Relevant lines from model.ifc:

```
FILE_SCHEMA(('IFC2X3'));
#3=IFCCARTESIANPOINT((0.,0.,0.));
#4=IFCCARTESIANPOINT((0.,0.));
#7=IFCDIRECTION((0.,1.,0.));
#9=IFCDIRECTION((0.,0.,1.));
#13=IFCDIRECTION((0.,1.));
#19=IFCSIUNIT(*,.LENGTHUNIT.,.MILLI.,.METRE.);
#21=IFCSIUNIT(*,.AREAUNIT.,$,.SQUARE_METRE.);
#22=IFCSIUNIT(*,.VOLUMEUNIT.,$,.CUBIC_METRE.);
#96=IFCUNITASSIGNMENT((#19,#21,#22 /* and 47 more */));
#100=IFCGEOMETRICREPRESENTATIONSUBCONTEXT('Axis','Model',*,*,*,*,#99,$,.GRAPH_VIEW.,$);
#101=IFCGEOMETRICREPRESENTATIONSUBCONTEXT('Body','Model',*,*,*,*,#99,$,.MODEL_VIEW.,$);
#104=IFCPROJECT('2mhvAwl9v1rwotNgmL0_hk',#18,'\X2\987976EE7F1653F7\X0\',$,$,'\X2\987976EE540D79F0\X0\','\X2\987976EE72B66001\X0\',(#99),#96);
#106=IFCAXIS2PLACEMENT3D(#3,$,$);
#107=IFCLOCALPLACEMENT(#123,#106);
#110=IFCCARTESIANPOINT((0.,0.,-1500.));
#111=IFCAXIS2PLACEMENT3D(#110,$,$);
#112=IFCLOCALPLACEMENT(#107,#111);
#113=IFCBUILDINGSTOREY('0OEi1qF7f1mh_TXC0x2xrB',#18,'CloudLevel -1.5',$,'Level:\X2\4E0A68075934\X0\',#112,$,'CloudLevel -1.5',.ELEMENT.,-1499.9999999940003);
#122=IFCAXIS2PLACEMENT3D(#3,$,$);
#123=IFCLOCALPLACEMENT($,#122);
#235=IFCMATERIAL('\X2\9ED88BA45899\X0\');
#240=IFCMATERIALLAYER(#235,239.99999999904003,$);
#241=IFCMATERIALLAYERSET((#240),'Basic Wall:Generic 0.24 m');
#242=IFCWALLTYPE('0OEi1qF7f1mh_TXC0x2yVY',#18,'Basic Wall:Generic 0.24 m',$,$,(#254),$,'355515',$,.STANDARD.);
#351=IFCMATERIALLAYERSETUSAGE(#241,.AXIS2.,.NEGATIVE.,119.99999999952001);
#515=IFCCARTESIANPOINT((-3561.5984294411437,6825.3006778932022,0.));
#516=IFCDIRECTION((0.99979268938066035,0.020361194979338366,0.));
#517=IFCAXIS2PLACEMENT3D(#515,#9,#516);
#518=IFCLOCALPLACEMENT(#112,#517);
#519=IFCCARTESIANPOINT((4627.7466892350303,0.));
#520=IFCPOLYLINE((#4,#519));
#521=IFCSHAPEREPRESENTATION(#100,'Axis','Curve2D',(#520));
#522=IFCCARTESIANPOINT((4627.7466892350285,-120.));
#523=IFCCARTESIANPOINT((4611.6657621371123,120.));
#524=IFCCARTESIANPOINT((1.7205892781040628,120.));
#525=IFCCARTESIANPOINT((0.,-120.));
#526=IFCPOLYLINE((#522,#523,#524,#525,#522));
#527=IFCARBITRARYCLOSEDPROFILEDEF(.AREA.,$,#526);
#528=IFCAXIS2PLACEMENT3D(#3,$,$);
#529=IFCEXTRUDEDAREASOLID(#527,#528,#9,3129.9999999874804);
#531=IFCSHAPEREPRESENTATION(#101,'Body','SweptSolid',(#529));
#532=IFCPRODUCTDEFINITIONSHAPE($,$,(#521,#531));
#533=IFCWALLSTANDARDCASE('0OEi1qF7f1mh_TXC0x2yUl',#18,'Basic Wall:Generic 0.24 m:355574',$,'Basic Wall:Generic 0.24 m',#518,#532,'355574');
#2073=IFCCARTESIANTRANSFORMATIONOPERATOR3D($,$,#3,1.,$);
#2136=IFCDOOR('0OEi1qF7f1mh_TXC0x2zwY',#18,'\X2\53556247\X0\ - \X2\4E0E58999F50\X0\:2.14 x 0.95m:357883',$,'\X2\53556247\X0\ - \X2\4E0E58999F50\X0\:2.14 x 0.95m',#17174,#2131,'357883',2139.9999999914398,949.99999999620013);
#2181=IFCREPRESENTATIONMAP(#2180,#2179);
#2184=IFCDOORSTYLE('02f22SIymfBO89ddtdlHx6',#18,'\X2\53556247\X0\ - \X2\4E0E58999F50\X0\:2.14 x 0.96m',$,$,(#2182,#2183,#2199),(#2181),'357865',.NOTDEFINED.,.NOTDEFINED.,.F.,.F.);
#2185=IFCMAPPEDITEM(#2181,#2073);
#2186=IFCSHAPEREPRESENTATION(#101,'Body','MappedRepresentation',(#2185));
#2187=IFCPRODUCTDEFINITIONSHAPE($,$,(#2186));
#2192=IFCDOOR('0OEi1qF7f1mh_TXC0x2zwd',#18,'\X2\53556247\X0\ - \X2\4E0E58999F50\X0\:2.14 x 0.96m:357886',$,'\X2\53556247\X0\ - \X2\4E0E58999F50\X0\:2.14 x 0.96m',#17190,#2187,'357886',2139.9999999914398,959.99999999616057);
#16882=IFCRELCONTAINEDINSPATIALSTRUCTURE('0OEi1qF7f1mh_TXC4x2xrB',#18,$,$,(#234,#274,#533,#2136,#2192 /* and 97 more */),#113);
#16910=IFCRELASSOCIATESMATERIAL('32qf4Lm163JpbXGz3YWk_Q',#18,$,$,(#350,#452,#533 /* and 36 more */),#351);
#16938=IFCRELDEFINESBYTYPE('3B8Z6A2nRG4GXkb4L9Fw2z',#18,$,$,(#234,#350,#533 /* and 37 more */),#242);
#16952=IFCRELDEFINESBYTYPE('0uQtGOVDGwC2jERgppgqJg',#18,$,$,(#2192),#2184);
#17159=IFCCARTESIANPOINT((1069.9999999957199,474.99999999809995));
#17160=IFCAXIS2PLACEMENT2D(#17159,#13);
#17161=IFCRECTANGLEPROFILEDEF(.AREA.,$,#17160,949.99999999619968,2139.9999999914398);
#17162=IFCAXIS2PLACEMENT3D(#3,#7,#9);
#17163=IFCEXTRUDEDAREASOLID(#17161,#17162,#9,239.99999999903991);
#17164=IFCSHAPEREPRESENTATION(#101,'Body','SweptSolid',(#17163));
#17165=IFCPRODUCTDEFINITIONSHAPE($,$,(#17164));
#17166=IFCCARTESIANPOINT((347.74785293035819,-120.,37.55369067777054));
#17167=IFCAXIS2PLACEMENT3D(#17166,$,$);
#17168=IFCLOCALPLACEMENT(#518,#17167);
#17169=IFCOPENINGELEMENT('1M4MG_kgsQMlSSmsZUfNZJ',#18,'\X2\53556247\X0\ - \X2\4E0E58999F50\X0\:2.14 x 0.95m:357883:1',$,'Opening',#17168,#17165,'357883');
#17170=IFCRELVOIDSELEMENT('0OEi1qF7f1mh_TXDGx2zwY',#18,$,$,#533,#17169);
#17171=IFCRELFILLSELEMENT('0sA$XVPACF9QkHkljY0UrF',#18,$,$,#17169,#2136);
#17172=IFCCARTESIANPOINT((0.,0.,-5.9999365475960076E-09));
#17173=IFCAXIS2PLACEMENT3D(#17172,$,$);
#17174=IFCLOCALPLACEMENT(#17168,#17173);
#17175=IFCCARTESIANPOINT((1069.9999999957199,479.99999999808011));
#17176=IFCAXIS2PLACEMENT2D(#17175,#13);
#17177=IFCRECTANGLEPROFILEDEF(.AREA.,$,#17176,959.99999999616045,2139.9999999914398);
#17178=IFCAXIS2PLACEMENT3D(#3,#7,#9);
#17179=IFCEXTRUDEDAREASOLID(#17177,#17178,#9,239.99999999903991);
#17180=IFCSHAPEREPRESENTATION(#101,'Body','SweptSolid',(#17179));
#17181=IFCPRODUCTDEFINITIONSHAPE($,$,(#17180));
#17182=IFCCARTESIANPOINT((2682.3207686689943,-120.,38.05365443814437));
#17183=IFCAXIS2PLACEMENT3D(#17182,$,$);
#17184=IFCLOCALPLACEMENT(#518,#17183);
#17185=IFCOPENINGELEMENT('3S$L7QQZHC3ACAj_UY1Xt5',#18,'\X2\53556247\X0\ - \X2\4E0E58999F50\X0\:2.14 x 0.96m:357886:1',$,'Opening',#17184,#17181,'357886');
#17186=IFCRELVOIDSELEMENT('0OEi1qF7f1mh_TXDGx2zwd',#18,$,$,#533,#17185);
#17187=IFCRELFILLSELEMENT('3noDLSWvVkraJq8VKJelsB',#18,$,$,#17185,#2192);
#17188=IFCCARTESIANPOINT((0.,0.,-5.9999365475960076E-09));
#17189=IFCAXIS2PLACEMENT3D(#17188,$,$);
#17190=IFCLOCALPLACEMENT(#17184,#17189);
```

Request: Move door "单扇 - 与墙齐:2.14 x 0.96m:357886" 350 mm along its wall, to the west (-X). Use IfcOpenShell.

```python
import ifcopenshell
import ifcopenshell.api.geometry
import ifcopenshell.util.placement

model = ifcopenshell.open("model.ifc")

door = model.by_id(2192)
opening = door.FillsVoids[0].RelatingOpeningElement
wall = opening.VoidsElements[0].RelatingBuildingElement

wall_matrix = ifcopenshell.util.placement.get_local_placement(wall.ObjectPlacement)
shift = wall_matrix[:3, 0] * -350.0
before = ifcopenshell.util.placement.get_local_placement(door.ObjectPlacement)[:3, 3].copy()

# The door is placed relative to its opening, so it follows when the opening moves.
matrix = ifcopenshell.util.placement.get_local_placement(opening.ObjectPlacement)
matrix[:3, 3] += shift
ifcopenshell.api.geometry.edit_object_placement(
    model, product=opening, matrix=matrix, is_si=False, should_transform_children=True
)

after = ifcopenshell.util.placement.get_local_placement(door.ObjectPlacement)[:3, 3]
print("door moved by", (after - before).round(3) + 0.0)

model.write("model_v2.ifc")
```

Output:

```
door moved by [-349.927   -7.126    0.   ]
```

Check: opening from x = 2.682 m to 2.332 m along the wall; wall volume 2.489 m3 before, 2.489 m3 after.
